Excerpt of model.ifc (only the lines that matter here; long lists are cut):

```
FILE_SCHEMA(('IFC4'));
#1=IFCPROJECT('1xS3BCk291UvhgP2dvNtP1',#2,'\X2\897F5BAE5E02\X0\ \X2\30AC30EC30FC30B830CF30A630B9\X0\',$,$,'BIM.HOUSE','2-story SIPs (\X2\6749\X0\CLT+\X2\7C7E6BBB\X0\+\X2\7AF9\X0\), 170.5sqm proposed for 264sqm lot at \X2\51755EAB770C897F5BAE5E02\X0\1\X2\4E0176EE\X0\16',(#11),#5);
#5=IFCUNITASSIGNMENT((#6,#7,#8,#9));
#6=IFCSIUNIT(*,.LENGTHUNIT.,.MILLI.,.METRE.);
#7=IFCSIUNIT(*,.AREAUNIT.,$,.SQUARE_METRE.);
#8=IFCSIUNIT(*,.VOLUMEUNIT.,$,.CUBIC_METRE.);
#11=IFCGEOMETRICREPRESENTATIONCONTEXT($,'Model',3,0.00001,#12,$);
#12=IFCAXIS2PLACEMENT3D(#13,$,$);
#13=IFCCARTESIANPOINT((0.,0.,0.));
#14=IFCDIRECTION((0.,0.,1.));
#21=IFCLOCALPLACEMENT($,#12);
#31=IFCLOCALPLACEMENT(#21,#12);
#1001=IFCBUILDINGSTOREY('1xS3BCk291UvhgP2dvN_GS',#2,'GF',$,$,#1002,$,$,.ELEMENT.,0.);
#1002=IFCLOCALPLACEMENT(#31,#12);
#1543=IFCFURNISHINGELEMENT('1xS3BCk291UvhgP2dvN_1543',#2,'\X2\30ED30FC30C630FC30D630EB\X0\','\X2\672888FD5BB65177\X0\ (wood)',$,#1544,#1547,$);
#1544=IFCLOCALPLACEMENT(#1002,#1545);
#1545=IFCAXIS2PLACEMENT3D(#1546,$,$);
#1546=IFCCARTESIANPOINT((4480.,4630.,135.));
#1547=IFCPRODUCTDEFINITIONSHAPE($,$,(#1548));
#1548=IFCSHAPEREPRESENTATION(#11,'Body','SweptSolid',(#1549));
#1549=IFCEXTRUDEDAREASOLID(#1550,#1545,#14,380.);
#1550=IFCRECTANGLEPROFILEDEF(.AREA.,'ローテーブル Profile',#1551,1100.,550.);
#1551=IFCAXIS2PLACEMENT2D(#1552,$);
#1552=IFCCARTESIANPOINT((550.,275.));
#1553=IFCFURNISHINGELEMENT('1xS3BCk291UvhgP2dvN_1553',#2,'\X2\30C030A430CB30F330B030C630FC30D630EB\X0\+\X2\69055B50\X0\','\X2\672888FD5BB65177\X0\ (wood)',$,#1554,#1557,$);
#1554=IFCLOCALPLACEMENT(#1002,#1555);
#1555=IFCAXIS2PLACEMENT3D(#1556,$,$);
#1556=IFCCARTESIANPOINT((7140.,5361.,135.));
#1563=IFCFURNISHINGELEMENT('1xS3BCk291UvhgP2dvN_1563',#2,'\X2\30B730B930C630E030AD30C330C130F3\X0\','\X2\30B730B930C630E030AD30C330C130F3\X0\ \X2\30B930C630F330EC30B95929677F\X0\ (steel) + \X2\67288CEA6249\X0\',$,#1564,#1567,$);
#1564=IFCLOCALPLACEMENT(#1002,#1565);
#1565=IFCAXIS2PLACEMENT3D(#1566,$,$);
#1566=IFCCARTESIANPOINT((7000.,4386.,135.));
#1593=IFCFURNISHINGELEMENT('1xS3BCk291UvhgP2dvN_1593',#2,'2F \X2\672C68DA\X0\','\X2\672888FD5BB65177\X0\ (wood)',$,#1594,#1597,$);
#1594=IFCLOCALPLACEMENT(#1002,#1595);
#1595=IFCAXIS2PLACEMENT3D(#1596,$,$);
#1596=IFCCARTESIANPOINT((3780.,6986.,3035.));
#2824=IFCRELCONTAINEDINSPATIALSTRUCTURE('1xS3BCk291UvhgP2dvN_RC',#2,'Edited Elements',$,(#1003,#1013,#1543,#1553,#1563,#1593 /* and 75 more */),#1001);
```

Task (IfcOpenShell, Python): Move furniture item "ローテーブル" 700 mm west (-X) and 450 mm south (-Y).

```python
import ifcopenshell
import ifcopenshell.api.geometry
import ifcopenshell.util.placement

model = ifcopenshell.open("model.ifc")

item = model.by_guid("1xS3BCk291UvhgP2dvN_1543")
matrix = ifcopenshell.util.placement.get_local_placement(item.ObjectPlacement)
matrix[0, 3] -= 700.0
matrix[1, 3] -= 450.0
ifcopenshell.api.geometry.edit_object_placement(model, product=item, matrix=matrix, is_si=False)

print(ifcopenshell.util.placement.get_local_placement(item.ObjectPlacement).round(3) + 0.0)

model.write("model_updated.ifc")
```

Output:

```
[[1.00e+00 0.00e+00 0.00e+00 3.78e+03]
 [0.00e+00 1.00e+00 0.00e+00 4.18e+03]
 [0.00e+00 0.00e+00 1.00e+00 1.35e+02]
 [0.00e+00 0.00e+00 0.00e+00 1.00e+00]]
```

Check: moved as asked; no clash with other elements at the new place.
